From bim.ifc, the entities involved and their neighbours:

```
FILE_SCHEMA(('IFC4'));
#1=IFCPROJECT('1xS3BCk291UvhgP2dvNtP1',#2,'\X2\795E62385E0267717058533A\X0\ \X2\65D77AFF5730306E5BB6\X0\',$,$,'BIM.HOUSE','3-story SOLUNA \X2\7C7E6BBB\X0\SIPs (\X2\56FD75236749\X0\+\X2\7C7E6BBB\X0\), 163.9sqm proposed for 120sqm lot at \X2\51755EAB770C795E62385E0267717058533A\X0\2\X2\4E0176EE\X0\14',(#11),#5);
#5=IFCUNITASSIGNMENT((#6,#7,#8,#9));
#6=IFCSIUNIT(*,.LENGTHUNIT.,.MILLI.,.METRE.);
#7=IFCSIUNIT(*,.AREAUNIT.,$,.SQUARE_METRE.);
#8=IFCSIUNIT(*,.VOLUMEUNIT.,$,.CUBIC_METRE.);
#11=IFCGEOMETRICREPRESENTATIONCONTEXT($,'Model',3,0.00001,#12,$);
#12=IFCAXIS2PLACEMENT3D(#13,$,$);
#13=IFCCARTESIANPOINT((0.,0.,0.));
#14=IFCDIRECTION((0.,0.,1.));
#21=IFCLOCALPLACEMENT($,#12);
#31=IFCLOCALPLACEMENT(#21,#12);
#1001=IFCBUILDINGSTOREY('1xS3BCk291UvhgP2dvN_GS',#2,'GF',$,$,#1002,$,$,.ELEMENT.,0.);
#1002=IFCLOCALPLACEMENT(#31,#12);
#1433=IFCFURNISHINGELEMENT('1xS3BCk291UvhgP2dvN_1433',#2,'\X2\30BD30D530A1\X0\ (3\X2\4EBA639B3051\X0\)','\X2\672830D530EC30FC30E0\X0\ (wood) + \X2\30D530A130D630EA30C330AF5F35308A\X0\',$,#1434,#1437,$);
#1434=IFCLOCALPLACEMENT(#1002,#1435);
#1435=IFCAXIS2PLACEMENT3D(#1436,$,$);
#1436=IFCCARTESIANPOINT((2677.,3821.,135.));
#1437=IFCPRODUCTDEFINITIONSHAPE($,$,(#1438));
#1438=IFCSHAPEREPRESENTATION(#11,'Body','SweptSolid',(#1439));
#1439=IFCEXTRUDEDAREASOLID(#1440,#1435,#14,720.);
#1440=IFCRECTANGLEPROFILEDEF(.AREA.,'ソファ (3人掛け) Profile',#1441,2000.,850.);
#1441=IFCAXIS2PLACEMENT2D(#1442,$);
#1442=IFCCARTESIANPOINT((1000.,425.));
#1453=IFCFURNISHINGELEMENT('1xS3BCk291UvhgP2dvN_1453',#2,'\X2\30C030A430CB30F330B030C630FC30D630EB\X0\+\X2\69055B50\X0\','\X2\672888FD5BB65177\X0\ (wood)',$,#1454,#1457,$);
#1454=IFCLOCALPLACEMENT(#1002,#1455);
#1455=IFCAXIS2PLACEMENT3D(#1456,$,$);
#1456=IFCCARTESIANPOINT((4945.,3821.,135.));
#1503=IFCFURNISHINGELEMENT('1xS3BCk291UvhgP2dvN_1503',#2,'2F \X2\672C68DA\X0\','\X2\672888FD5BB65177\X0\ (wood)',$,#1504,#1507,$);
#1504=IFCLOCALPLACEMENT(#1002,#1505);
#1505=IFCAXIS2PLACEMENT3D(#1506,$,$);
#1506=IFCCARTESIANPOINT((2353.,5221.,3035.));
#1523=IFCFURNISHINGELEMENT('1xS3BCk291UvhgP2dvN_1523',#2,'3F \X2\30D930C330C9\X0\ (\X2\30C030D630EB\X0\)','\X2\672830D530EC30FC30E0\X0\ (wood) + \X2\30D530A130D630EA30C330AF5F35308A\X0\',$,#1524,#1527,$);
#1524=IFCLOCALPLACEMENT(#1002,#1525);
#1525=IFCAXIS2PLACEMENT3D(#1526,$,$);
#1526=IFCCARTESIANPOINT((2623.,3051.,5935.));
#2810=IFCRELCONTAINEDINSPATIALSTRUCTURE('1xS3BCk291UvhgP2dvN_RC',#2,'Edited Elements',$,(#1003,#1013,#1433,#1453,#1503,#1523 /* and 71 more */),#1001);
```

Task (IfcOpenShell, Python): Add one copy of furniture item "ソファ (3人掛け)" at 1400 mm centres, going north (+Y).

```python
import numpy as np
import ifcopenshell
import ifcopenshell.api.geometry
import ifcopenshell.api.root
import ifcopenshell.util.element
import ifcopenshell.util.placement
import ifcopenshell.util.unit

model = ifcopenshell.open("bim.ifc")
unit_scale = ifcopenshell.util.unit.calculate_unit_scale(model)


def reuse_history(source, copy):
    """copy_class also copies each property set's owner history, people and application; keep the originals."""
    for rel in copy.IsDefinedBy:
        if rel.is_a("IfcRelDefinesByProperties") and (history := rel.RelatingPropertyDefinition.OwnerHistory):
            rel.RelatingPropertyDefinition.OwnerHistory = source.OwnerHistory
            ifcopenshell.util.element.remove_deep2(model, history)


source = model.by_guid("1xS3BCk291UvhgP2dvN_1433")
base = ifcopenshell.util.placement.get_local_placement(source.ObjectPlacement)
step = np.array([0.0, 1.0, 0.0]) * 1.4 / unit_scale

for i in range(1, 2):
    copy = ifcopenshell.api.root.copy_class(model, product=source)
    copy.Representation = ifcopenshell.util.element.copy_deep(
        model, source.Representation, exclude=["IfcGeometricRepresentationContext", "IfcRepresentationMap"]
    )
    reuse_history(source, copy)
    matrix = base.copy()
    matrix[:3, 3] += i * step
    print("added at", matrix[:3, 3].round(3) + 0.0)
    ifcopenshell.api.geometry.edit_object_placement(model, product=copy, matrix=matrix, is_si=False)

model.write("bim_edited.ifc")
```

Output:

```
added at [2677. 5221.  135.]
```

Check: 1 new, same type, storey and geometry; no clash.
